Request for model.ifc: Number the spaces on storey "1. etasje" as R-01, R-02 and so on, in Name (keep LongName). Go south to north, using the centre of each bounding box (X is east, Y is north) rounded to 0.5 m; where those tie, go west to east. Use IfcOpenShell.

First a look at what the model holds.

```python
import ifcopenshell
import ifcopenshell.util.element
import ifcopenshell.util.placement

model = ifcopenshell.open("model.ifc")
print(model.schema)
storey = next(s for s in model.by_type("IfcBuildingStorey") if s.Name == "1. etasje")
spaces = [e for e in ifcopenshell.util.element.get_decomposition(storey) if e.is_a("IfcSpace")]
for e in sorted(spaces, key=lambda e: e.id()):
    origin = ifcopenshell.util.placement.get_local_placement(e.ObjectPlacement)[:3, 3]
    print(e.id(), e.Name, e.LongName, origin.round(2) + 0.0, sep=" | ")
```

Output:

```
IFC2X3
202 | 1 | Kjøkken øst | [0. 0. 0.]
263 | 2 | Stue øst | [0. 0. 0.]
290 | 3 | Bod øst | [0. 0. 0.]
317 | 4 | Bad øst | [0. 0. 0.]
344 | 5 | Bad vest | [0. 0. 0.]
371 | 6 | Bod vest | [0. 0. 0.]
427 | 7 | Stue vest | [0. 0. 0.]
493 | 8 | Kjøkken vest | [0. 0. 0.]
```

```python
import ifcopenshell
import ifcopenshell.geom
import ifcopenshell.util.element
import ifcopenshell.util.shape

model = ifcopenshell.open("model.ifc")
settings = ifcopenshell.geom.settings()
settings.set("use-world-coords", True)


def centre(element):
    shape = ifcopenshell.geom.create_shape(settings, element)
    return ifcopenshell.util.shape.get_bbox_centroid(shape.geometry)


storey = next(s for s in model.by_type("IfcBuildingStorey") if s.Name == "1. etasje")
spaces = [e for e in ifcopenshell.util.element.get_decomposition(storey) if e.is_a("IfcSpace")]

# Insertion points can sit at a corner or the storey origin, so sort by the geometry (in metres).
centres = {e: centre(e) for e in spaces}
spaces.sort(key=lambda e: (round(centres[e][1] / 0.5), centres[e][0]))

for i, e in enumerate(spaces, start=1):
    number = f"R-{i:02d}"
    e.Name = number
    print(e.id(), number)

model.write("model_rev.ifc")
```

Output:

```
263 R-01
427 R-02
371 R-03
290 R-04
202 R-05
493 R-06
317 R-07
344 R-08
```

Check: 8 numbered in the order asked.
